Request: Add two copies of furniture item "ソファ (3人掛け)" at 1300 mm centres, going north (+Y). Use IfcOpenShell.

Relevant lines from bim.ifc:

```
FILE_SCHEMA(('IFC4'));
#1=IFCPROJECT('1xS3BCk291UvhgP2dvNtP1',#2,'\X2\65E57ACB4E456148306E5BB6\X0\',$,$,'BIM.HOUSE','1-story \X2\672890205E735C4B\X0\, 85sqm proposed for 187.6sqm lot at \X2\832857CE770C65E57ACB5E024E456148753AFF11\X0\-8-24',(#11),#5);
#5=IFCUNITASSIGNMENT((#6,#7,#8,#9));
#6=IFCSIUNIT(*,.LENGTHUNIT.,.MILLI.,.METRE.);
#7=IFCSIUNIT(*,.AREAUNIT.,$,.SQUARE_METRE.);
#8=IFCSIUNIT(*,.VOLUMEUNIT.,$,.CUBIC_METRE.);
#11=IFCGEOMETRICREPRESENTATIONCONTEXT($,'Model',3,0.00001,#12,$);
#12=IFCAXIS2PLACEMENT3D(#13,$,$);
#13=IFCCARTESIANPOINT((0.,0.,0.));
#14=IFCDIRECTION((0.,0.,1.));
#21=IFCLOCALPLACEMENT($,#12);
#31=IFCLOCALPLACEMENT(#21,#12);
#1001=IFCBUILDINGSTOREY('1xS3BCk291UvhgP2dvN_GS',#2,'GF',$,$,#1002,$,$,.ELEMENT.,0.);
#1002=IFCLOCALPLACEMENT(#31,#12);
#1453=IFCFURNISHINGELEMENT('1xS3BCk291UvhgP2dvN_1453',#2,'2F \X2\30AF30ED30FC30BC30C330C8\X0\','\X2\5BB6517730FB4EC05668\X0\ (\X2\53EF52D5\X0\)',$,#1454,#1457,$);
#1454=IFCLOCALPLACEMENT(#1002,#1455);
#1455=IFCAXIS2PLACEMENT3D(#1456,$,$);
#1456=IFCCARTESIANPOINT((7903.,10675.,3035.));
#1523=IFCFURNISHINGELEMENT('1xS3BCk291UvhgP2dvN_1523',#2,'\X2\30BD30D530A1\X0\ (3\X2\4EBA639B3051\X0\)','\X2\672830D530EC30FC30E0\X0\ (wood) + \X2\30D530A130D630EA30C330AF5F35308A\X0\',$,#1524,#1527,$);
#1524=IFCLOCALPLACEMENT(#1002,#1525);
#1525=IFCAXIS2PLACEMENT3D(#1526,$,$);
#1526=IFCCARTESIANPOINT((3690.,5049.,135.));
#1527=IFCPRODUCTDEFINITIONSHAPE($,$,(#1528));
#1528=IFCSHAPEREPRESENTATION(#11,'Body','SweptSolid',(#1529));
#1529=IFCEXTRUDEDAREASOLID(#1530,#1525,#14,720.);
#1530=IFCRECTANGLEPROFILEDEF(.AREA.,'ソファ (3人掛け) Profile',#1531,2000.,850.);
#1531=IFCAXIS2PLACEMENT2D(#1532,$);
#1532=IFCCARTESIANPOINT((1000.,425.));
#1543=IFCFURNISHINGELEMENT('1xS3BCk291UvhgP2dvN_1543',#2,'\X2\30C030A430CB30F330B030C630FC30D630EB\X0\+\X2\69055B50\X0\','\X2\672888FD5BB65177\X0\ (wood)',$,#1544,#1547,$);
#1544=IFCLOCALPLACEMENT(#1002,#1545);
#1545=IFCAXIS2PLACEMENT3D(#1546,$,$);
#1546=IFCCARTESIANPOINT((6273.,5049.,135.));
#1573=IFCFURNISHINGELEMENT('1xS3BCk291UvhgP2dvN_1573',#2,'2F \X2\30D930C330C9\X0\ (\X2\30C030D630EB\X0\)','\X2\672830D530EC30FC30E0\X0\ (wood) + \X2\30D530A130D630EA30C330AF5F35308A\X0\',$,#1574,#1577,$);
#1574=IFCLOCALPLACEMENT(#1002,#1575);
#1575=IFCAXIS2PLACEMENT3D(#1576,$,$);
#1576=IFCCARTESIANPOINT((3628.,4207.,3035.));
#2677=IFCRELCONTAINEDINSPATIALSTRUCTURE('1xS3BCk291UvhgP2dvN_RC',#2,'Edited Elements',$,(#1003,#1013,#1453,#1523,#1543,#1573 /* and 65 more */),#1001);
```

```python
import numpy as np
import ifcopenshell
import ifcopenshell.api.geometry
import ifcopenshell.api.root
import ifcopenshell.util.element
import ifcopenshell.util.placement

model = ifcopenshell.open("bim.ifc")


def reuse_history(source, copy):
    """copy_class also copies each property set's owner history, people and application; keep the originals."""
    for rel in copy.IsDefinedBy:
        if rel.is_a("IfcRelDefinesByProperties") and (history := rel.RelatingPropertyDefinition.OwnerHistory):
            rel.RelatingPropertyDefinition.OwnerHistory = source.OwnerHistory
            ifcopenshell.util.element.remove_deep2(model, history)


source = model.by_guid("1xS3BCk291UvhgP2dvN_1523")
base = ifcopenshell.util.placement.get_local_placement(source.ObjectPlacement)
step = np.array([0.0, 1.0, 0.0]) * 1300.0

for i in range(1, 3):
    copy = ifcopenshell.api.root.copy_class(model, product=source)
    copy.Representation = ifcopenshell.util.element.copy_deep(
        model, source.Representation, exclude=["IfcGeometricRepresentationContext", "IfcRepresentationMap"]
    )
    reuse_history(source, copy)
    matrix = base.copy()
    matrix[:3, 3] += i * step
    print("added at", matrix[:3, 3].round(3) + 0.0)
    ifcopenshell.api.geometry.edit_object_placement(model, product=copy, matrix=matrix, is_si=False)

model.write("bim_rev.ifc")
```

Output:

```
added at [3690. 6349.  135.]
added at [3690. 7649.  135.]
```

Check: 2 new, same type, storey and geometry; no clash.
